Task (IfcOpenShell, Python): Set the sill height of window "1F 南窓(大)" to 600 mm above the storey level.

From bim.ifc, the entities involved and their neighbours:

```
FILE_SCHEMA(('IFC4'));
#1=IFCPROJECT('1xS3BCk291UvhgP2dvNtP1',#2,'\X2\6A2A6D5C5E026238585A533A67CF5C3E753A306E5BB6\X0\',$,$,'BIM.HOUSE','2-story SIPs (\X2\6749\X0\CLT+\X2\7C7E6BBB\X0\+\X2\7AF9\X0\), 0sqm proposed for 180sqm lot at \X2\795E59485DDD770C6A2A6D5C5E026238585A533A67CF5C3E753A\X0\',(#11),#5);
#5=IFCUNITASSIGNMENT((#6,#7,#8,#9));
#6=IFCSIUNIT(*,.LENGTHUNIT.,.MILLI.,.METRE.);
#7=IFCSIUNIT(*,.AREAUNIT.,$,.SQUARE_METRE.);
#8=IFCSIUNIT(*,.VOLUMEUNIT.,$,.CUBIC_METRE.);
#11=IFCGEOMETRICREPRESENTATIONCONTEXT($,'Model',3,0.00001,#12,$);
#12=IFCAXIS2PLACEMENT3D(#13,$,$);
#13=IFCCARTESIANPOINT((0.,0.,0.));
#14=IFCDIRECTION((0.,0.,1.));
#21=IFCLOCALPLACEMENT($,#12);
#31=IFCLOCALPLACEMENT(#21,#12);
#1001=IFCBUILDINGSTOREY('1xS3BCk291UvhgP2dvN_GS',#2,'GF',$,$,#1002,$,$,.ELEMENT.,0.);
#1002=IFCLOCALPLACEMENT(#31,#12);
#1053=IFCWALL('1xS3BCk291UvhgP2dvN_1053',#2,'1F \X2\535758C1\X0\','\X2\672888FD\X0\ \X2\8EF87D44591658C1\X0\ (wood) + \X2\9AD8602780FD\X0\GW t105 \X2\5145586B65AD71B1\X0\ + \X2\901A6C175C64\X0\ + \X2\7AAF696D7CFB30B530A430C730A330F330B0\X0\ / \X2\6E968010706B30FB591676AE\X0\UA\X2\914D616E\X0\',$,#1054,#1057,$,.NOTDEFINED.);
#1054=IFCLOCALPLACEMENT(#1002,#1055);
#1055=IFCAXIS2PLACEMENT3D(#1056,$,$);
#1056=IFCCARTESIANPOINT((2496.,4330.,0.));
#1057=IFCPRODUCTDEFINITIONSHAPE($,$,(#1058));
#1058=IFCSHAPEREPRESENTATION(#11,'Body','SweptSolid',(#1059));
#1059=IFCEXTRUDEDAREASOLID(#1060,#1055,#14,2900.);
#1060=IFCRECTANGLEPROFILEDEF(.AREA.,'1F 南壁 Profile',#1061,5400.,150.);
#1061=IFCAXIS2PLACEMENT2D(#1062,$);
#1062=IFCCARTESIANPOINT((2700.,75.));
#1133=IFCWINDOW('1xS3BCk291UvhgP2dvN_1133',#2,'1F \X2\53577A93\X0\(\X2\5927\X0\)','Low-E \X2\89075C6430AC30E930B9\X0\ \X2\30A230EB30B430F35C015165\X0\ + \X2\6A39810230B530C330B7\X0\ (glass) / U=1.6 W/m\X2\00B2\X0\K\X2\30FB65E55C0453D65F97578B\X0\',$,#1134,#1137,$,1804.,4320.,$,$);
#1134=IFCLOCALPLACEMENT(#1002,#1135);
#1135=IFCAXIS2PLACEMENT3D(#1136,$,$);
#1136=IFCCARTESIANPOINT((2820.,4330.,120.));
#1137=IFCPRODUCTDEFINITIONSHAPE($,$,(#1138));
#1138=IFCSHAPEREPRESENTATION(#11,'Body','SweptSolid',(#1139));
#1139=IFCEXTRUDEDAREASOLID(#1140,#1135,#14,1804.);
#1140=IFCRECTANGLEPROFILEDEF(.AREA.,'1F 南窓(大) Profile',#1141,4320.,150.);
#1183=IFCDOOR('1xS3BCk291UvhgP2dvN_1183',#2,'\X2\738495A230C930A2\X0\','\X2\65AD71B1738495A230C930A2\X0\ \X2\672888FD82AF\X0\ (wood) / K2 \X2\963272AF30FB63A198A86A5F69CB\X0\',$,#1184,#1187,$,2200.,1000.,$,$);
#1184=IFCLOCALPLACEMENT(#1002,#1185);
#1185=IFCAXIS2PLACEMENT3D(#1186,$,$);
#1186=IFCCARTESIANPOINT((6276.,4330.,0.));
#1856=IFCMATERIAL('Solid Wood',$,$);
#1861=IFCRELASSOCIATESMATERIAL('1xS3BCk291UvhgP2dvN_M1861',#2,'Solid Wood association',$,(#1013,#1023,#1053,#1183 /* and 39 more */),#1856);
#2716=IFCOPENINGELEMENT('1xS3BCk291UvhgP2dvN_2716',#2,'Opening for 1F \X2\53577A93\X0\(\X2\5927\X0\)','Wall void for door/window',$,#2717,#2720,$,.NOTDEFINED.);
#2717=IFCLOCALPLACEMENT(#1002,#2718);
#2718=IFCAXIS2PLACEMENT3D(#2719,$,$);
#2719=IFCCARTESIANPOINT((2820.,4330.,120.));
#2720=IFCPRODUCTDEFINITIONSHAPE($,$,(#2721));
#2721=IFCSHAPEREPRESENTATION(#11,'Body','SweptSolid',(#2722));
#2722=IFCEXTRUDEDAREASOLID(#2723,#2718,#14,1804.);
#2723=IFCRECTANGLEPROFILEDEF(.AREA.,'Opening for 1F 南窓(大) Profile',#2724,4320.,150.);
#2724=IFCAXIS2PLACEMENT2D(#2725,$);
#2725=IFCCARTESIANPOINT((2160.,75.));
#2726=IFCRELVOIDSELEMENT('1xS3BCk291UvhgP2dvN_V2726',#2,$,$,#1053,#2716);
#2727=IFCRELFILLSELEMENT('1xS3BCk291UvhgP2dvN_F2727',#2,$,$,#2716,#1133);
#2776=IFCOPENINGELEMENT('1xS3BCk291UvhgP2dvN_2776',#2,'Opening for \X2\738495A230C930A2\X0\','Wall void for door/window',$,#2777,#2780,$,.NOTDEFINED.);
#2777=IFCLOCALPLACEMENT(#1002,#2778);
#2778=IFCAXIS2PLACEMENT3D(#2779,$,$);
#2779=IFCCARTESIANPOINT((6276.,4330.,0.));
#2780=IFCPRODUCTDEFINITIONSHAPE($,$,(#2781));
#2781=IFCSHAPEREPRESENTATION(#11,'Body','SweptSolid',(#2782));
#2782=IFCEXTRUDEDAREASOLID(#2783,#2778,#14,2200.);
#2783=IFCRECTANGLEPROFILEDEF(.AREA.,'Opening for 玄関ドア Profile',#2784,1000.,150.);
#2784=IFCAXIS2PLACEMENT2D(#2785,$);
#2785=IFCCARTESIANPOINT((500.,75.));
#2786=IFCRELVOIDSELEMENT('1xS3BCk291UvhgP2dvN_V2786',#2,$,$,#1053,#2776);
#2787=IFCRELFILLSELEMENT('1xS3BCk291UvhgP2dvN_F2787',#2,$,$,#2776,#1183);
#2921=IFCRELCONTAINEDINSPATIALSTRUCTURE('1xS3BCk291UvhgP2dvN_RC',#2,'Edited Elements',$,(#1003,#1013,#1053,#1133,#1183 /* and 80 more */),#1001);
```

```python
import numpy as np
import ifcopenshell
import ifcopenshell.api.geometry
import ifcopenshell.geom
import ifcopenshell.util.element
import ifcopenshell.util.placement
import ifcopenshell.util.shape
import ifcopenshell.util.unit

model = ifcopenshell.open("bim.ifc")
unit_scale = ifcopenshell.util.unit.calculate_unit_scale(model)

window = model.by_id(1133)
opening = window.FillsVoids[0].RelatingOpeningElement
storey = ifcopenshell.util.element.get_container(window, ifc_class="IfcBuildingStorey")
level = ifcopenshell.util.placement.get_local_placement(storey.ObjectPlacement)[2, 3]

# The opening's origin need not be at the sill, so measure its lowest point.
shape = ifcopenshell.geom.create_shape(ifcopenshell.geom.settings(), opening)
bottom = ifcopenshell.util.shape.get_shape_bottom_elevation(shape, shape.geometry) / unit_scale
dz = level + 600.0 - bottom

shift = np.array([0.0, 0.0, dz])
# The window is not placed relative to its opening, so move both.
for product in (opening, window):
    matrix = ifcopenshell.util.placement.get_local_placement(product.ObjectPlacement)
    matrix[:3, 3] += shift
    ifcopenshell.api.geometry.edit_object_placement(model, product=product, matrix=matrix, is_si=False)

print(f"moved by {dz * unit_scale:+.3f} m")

model.write("bim-out.ifc")
```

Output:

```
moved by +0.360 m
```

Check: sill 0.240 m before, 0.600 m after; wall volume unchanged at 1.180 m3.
